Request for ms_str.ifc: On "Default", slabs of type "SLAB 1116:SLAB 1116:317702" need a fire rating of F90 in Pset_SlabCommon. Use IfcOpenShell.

First a look at what the model holds.

```python
import ifcopenshell
import ifcopenshell.util.element

model = ifcopenshell.open("ms_str.ifc")
print(model.schema)
storey = next(s for s in model.by_type("IfcBuildingStorey") if s.Name == "Default")
slabs = [e for e in ifcopenshell.util.element.get_decomposition(storey) if e.is_a("IfcSlab")]
seen = {}
for e in slabs:
    element_type = ifcopenshell.util.element.get_type(e)
    key = (element_type.Name if element_type != e and element_type else None, ifcopenshell.util.element.get_pset(e, "Pset_SlabCommon", "FireRating"))
    seen[key] = seen.get(key, 0) + 1
for (name, value), count in sorted(seen.items(), key=str):
    print(count, "x", name, "|", value)
```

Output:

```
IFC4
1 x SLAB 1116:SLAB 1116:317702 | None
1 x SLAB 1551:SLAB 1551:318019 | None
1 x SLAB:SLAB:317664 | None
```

```python
import ifcopenshell
import ifcopenshell.api.pset
import ifcopenshell.util.element

model = ifcopenshell.open("ms_str.ifc")

storey = next(s for s in model.by_type("IfcBuildingStorey") if s.Name == "Default")
slabs = [e for e in ifcopenshell.util.element.get_decomposition(storey) if e.is_a("IfcSlab")]

count = 0
for e in slabs:
    element_type = ifcopenshell.util.element.get_type(e)
    if element_type in (None, e) or element_type.Name != "SLAB 1116:SLAB 1116:317702":
        continue
    # add_pset returns the element's existing set when there is one.
    pset = ifcopenshell.api.pset.add_pset(model, product=e, name="Pset_SlabCommon")
    ifcopenshell.api.pset.edit_pset(model, pset=pset, properties={"FireRating": "F90"})
    count += 1

print(count, "slabs updated")

model.write("ms_str-out.ifc")
```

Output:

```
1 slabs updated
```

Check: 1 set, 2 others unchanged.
